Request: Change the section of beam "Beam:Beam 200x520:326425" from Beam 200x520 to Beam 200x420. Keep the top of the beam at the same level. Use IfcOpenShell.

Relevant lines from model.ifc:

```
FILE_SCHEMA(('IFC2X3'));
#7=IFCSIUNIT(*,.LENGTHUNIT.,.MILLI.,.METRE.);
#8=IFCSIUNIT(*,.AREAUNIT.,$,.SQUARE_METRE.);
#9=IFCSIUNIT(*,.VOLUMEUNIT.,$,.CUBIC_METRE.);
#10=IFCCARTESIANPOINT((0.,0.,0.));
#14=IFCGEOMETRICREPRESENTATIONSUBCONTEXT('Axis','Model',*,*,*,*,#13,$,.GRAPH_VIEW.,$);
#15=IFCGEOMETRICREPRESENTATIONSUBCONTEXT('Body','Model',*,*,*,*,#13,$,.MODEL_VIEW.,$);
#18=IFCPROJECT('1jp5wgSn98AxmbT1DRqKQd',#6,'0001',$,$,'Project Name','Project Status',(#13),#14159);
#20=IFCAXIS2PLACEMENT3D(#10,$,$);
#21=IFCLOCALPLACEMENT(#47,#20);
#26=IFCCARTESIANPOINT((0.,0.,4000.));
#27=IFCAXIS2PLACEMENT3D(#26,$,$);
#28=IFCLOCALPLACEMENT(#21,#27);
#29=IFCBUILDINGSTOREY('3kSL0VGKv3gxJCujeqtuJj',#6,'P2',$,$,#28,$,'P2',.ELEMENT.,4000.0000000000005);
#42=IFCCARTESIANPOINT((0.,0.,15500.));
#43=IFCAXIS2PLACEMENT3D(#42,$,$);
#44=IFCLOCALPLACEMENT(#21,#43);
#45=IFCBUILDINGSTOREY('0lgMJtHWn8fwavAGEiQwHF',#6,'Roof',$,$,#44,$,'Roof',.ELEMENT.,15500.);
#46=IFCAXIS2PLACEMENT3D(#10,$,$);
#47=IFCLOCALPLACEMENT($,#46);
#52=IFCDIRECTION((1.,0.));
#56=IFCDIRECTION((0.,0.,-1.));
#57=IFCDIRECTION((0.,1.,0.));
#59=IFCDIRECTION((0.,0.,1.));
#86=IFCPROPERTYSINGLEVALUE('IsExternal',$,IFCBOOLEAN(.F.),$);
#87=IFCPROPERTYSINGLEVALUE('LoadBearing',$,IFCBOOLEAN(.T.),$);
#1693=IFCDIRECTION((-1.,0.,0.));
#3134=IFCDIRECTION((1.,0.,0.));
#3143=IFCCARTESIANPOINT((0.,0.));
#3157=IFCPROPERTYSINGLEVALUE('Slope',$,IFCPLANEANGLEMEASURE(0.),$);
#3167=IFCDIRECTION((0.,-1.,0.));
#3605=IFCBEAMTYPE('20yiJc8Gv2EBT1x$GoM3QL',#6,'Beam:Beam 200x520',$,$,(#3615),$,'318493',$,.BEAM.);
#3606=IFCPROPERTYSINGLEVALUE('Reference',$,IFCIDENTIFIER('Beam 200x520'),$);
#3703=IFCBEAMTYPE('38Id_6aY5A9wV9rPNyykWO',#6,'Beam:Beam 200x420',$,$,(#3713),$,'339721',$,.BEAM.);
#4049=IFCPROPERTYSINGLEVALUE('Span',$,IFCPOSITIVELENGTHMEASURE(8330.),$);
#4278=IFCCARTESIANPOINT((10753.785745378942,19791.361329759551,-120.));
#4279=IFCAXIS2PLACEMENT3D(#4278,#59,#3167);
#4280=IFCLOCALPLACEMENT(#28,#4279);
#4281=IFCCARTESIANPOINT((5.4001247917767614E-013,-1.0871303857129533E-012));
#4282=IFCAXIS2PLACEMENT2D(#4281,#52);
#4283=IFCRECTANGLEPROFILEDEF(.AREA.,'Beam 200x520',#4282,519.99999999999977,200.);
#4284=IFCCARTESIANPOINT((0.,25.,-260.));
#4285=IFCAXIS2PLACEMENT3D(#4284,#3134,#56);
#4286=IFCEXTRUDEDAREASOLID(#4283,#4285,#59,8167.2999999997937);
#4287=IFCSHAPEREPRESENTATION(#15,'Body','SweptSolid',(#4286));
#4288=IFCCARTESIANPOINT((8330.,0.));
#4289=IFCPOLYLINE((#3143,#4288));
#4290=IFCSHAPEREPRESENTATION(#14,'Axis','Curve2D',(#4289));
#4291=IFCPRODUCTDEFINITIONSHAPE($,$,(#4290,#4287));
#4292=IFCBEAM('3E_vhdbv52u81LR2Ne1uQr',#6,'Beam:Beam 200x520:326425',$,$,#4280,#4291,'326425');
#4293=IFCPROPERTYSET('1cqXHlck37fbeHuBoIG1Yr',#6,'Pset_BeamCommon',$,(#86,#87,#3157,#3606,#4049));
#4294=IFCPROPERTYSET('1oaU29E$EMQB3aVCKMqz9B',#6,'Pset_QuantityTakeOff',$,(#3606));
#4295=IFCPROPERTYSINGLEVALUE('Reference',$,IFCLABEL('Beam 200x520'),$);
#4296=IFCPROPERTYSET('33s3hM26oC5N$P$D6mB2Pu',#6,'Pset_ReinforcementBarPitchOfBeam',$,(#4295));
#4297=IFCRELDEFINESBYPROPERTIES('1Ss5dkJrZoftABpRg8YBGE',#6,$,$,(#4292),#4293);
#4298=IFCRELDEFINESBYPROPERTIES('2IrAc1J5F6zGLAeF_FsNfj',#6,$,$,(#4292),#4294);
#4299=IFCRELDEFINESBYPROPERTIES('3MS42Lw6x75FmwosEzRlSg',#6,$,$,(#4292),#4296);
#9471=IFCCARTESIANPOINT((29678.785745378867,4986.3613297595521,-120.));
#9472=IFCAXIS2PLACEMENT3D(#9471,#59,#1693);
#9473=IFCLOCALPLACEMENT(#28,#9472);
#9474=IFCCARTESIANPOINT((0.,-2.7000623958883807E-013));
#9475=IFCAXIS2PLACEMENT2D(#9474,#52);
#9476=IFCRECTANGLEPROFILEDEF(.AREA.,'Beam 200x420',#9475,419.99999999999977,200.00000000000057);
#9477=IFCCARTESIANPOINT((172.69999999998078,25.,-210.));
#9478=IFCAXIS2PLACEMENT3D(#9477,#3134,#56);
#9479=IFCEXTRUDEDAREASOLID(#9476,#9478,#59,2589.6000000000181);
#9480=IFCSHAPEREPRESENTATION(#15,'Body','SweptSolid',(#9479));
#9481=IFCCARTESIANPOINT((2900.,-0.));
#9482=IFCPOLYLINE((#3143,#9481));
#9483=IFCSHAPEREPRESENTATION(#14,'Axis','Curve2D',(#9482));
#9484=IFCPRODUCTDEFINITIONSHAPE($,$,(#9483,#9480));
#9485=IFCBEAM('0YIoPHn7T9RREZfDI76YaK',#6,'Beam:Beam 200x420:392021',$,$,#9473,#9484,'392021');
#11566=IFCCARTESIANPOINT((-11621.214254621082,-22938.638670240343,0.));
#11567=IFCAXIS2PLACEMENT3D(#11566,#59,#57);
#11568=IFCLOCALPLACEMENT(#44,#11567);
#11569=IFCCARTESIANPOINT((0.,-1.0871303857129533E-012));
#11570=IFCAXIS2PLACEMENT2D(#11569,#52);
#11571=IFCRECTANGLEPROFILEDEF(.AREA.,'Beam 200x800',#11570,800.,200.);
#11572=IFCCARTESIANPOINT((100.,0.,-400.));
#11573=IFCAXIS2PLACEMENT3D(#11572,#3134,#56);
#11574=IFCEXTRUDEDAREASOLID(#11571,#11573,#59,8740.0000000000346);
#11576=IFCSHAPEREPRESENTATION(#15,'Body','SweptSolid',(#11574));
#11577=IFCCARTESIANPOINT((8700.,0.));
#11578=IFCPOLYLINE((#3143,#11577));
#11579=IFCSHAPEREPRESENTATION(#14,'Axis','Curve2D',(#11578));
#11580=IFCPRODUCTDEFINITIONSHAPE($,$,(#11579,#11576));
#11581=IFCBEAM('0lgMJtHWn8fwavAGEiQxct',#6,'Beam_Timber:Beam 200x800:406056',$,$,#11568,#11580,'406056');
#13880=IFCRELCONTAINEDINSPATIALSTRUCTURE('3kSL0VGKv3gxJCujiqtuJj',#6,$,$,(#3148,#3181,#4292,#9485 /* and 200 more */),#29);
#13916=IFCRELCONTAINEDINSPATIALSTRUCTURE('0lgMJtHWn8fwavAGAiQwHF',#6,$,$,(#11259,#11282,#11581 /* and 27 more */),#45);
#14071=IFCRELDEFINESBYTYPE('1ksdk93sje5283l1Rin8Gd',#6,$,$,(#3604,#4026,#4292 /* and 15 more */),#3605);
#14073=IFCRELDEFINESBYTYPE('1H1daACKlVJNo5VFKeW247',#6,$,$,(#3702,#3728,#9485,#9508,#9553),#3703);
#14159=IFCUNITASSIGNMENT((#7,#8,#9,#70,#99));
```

```python
import ifcopenshell
import ifcopenshell.api.pset
import ifcopenshell.api.type
import ifcopenshell.util.element
import ifcopenshell.util.representation

model = ifcopenshell.open("model.ifc")

member = model.by_guid("3E_vhdbv52u81LR2Ne1uQr")
source = next(p for p in model.by_type("IfcRectangleProfileDef") if p.ProfileName == "Beam 200x420")

body = ifcopenshell.util.representation.get_representation(member, "Model", "Body")
solid = body.Items[0]
old_profile = solid.SweptArea

# Copy the section's sizes but keep this member's own profile position.
profile = ifcopenshell.util.element.copy(model, source)
# Profiles are centred, so shift by half the change in depth to hold the top.
shift = (old_profile.XDim - profile.XDim) / 2
x, y = old_profile.Position.Location.Coordinates
up = (-1.0, 0.0)  # upwards, in the solid's own plane
location = model.createIfcCartesianPoint((x + up[0] * shift, y + up[1] * shift))
profile.Position = model.createIfcAxis2Placement2D(location, old_profile.Position.RefDirection)
solid.SweptArea = profile
if not model.get_total_inverses(old_profile):
    ifcopenshell.util.element.remove_deep2(model, old_profile)

new_type = model.by_id(3703)
ifcopenshell.api.type.assign_type(
    model, related_objects=[member], relating_type=new_type, should_map_representations=False
)
member.Name = member.Name.replace("Beam 200x520", "Beam 200x420")
pset = model.by_id(ifcopenshell.util.element.get_pset(member, "Pset_BeamCommon", should_inherit=False)["id"])
ifcopenshell.api.pset.edit_pset(model, pset=pset, properties={"Reference": "Beam 200x420"})
pset = model.by_id(ifcopenshell.util.element.get_pset(member, "Pset_QuantityTakeOff", should_inherit=False)["id"])
ifcopenshell.api.pset.edit_pset(model, pset=pset, properties={"Reference": "Beam 200x420"})
pset = model.by_id(ifcopenshell.util.element.get_pset(member, "Pset_ReinforcementBarPitchOfBeam", should_inherit=False)["id"])
ifcopenshell.api.pset.edit_pset(model, pset=pset, properties={"Reference": "Beam 200x420"})

print(solid.SweptArea)

model.write("model_edited.ifc")
```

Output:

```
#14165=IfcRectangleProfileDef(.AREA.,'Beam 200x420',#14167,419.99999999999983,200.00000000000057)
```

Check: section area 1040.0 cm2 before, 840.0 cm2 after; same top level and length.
